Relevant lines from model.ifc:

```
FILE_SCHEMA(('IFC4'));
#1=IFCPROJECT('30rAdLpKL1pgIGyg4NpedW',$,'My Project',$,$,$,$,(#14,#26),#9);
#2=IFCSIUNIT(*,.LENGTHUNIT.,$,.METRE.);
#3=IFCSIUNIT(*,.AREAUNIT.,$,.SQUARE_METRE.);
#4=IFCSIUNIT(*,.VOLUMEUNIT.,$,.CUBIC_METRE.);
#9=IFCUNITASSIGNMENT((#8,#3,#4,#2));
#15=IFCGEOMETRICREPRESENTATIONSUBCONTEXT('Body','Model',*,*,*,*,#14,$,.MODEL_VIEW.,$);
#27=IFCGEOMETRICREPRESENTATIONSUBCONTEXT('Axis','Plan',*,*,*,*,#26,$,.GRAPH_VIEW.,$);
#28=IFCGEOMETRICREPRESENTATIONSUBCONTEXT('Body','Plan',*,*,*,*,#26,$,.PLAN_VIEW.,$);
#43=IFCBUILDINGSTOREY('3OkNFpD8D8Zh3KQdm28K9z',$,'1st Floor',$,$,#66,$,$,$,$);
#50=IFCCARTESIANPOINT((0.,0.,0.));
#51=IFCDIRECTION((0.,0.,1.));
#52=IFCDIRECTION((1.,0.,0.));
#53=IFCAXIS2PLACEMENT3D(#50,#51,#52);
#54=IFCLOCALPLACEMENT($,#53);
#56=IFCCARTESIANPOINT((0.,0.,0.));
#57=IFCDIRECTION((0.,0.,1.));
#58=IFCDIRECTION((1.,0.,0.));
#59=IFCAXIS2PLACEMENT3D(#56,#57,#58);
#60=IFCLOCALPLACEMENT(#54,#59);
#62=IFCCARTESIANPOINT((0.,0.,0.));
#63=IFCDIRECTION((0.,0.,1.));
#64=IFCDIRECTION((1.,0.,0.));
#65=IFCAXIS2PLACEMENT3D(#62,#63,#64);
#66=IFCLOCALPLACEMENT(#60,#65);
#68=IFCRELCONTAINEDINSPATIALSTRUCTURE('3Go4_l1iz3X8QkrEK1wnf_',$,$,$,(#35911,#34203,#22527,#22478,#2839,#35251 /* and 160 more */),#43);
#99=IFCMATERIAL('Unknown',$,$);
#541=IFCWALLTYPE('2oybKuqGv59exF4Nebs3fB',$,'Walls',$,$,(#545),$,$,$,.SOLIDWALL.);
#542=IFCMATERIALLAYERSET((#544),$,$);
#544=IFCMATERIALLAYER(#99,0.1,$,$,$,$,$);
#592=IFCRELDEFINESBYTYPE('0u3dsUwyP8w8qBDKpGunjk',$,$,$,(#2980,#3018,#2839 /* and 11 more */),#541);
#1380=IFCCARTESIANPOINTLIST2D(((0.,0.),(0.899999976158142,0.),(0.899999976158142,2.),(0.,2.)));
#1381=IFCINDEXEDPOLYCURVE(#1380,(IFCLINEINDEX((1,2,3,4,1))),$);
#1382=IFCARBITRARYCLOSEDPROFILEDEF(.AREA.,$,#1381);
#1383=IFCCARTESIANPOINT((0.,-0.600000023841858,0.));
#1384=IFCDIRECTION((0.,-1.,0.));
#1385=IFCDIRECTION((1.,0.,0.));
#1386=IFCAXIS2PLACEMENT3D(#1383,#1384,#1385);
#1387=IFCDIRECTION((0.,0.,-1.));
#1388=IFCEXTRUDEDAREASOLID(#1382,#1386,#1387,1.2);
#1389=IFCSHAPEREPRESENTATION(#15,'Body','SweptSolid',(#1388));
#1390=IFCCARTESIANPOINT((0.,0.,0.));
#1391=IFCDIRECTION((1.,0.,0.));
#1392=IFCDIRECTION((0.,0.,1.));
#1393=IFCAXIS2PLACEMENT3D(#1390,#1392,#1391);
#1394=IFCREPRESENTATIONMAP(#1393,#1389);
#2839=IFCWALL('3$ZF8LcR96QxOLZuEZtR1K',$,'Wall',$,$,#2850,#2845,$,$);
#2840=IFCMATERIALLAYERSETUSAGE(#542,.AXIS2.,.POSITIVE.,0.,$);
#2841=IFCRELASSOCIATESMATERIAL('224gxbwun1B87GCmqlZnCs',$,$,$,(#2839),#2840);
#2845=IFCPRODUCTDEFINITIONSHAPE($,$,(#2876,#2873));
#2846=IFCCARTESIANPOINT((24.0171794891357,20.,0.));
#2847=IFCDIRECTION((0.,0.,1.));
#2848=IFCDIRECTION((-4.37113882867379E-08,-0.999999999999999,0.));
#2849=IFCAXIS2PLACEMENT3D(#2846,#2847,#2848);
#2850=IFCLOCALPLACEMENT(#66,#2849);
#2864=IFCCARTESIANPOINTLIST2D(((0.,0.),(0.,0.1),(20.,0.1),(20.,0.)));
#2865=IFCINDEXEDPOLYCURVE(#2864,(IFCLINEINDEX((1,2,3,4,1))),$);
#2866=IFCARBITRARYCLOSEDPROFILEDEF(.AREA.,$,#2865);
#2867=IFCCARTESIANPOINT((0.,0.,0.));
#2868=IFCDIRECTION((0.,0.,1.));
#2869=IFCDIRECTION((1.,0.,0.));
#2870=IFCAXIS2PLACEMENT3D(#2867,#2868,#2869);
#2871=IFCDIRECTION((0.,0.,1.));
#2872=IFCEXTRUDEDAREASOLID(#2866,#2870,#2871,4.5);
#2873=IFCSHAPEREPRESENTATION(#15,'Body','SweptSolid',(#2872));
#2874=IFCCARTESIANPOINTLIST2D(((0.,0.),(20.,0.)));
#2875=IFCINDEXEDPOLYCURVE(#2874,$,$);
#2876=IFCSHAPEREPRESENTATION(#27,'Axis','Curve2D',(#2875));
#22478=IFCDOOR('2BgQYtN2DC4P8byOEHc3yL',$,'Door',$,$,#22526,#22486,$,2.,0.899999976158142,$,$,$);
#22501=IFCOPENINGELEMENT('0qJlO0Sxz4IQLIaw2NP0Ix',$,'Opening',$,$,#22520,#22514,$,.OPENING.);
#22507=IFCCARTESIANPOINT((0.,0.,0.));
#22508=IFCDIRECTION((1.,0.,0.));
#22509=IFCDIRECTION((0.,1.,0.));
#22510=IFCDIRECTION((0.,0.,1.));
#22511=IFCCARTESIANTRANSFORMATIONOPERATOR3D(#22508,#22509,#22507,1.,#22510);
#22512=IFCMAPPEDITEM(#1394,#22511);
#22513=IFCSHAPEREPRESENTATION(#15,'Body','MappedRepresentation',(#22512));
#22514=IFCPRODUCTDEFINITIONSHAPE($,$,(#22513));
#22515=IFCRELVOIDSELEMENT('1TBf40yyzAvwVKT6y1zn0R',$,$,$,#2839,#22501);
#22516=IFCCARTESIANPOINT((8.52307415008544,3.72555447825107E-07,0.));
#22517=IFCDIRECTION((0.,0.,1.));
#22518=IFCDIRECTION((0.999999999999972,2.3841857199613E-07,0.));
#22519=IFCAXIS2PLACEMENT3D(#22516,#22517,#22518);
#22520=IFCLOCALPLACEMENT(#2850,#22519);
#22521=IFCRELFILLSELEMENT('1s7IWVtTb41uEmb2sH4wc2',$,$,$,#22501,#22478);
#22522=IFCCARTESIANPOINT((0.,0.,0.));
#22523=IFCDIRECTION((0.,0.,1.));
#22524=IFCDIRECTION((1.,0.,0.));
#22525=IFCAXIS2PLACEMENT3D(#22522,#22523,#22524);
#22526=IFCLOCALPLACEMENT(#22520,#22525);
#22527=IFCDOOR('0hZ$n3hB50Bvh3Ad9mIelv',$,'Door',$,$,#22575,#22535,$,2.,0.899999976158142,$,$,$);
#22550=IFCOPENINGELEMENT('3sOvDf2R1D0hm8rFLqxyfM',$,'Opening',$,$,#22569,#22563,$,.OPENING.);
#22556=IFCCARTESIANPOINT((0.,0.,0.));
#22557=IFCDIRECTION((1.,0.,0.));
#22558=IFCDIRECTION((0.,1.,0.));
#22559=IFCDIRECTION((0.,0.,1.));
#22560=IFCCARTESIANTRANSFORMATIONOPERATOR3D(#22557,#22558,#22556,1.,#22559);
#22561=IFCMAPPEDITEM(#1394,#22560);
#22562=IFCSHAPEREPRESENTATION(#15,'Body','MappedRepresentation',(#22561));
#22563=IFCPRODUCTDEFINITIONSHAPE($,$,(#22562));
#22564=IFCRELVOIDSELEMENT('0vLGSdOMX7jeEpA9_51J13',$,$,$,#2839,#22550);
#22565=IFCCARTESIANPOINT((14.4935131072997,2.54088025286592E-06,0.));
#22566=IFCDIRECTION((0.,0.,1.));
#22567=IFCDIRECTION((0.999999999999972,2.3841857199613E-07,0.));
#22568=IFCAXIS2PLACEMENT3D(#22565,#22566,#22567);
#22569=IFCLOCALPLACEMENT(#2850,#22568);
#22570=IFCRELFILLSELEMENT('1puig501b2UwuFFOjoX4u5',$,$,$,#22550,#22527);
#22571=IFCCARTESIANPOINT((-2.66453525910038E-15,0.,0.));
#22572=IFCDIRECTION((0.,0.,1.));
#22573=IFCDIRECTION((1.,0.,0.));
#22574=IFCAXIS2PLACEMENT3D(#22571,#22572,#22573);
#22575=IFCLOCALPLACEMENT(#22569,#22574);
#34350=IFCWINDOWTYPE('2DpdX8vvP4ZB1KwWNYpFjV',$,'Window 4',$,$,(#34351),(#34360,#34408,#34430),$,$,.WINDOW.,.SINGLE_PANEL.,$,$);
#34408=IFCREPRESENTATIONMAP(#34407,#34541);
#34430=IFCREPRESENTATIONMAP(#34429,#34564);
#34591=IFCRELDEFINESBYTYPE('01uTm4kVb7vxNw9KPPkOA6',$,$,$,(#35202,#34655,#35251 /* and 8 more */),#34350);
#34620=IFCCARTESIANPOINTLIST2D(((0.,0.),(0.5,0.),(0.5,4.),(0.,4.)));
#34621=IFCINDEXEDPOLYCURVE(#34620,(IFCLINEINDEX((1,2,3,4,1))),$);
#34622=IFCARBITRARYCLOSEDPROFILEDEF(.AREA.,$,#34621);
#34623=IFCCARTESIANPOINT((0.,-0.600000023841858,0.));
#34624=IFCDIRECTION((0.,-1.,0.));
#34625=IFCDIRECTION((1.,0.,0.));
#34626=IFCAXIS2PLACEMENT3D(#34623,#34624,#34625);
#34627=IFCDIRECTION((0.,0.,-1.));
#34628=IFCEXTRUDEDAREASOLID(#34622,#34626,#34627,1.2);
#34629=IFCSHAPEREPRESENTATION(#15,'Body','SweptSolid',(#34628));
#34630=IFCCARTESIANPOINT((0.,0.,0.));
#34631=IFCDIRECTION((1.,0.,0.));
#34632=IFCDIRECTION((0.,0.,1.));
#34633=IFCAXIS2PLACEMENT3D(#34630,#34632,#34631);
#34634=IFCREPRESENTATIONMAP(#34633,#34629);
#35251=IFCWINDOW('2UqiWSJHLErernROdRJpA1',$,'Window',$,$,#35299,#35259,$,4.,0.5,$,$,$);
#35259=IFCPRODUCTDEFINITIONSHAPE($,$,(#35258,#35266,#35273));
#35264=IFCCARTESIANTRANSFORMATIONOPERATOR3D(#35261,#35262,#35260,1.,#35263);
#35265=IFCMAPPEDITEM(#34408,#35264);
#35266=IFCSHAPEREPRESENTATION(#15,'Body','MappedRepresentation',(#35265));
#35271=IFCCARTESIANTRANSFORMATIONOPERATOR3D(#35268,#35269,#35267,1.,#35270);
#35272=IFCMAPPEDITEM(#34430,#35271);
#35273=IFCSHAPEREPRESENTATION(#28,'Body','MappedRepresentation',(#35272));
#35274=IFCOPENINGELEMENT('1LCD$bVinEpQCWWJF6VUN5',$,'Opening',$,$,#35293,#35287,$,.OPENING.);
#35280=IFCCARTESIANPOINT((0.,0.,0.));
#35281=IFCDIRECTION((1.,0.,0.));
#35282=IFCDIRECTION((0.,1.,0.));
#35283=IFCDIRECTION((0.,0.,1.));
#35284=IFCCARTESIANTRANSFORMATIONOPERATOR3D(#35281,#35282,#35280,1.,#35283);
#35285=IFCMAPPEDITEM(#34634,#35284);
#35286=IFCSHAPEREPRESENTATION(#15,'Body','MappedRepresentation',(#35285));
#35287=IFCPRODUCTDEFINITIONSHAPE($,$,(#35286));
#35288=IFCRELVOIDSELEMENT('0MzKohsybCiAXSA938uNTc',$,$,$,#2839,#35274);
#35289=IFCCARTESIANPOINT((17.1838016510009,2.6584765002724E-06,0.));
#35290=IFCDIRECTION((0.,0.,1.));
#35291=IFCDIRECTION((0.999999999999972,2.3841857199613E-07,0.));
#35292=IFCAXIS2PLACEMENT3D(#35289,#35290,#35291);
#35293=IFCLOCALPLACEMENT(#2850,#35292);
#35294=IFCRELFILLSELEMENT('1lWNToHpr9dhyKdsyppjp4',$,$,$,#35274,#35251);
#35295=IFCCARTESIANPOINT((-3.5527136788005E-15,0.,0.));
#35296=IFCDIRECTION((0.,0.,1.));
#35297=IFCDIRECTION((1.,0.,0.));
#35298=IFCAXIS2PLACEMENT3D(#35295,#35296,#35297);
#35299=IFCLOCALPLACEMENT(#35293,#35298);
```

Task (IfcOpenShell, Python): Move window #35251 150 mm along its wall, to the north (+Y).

```python
import ifcopenshell
import ifcopenshell.api.geometry
import ifcopenshell.util.placement
import ifcopenshell.util.unit

model = ifcopenshell.open("model.ifc")
unit_scale = ifcopenshell.util.unit.calculate_unit_scale(model)

window = model.by_guid("2UqiWSJHLErernROdRJpA1")
opening = window.FillsVoids[0].RelatingOpeningElement
wall = opening.VoidsElements[0].RelatingBuildingElement

wall_matrix = ifcopenshell.util.placement.get_local_placement(wall.ObjectPlacement)
shift = wall_matrix[:3, 0] * -0.15 / unit_scale
before = ifcopenshell.util.placement.get_local_placement(window.ObjectPlacement)[:3, 3].copy()

# The window is placed relative to its opening, so it follows when the opening moves.
matrix = ifcopenshell.util.placement.get_local_placement(opening.ObjectPlacement)
matrix[:3, 3] += shift
ifcopenshell.api.geometry.edit_object_placement(
    model, product=opening, matrix=matrix, is_si=False, should_transform_children=True
)

after = ifcopenshell.util.placement.get_local_placement(window.ObjectPlacement)[:3, 3]
print("window moved by", (after - before).round(3) + 0.0)

model.write("model_rev.ifc")
```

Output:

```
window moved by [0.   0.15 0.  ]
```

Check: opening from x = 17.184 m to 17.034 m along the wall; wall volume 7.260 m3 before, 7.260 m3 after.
